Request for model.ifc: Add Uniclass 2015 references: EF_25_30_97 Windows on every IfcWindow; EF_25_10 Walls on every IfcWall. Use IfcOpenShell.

First a look at what the model holds.

```python
import ifcopenshell

model = ifcopenshell.open("model.ifc")
print(model.schema)
print("classifications:", [c.Name for c in model.by_type("IfcClassification")])
for ifc_class in ("IfcDoor", "IfcRoof", "IfcStair", "IfcWall", "IfcWindow"):
    print(ifc_class, len(model.by_type(ifc_class)))
```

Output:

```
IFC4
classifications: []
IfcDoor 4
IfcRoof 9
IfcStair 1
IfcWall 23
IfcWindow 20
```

```python
import ifcopenshell
import ifcopenshell.api.classification

model = ifcopenshell.open("model.ifc")

system = ifcopenshell.api.classification.add_classification(model, classification="Uniclass 2015")

codes = {
    "IfcWindow": ("EF_25_30_97", "Windows"),
    "IfcWall": ("EF_25_10", "Walls"),
}
for ifc_class, (code, name) in codes.items():
    products = model.by_type(ifc_class)
    ifcopenshell.api.classification.add_reference(
        model, products=products, classification=system, identification=code, name=name
    )
    print(code, len(products))

model.write("model_edited.ifc")
```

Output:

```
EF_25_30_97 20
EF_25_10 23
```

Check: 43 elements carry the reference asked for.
